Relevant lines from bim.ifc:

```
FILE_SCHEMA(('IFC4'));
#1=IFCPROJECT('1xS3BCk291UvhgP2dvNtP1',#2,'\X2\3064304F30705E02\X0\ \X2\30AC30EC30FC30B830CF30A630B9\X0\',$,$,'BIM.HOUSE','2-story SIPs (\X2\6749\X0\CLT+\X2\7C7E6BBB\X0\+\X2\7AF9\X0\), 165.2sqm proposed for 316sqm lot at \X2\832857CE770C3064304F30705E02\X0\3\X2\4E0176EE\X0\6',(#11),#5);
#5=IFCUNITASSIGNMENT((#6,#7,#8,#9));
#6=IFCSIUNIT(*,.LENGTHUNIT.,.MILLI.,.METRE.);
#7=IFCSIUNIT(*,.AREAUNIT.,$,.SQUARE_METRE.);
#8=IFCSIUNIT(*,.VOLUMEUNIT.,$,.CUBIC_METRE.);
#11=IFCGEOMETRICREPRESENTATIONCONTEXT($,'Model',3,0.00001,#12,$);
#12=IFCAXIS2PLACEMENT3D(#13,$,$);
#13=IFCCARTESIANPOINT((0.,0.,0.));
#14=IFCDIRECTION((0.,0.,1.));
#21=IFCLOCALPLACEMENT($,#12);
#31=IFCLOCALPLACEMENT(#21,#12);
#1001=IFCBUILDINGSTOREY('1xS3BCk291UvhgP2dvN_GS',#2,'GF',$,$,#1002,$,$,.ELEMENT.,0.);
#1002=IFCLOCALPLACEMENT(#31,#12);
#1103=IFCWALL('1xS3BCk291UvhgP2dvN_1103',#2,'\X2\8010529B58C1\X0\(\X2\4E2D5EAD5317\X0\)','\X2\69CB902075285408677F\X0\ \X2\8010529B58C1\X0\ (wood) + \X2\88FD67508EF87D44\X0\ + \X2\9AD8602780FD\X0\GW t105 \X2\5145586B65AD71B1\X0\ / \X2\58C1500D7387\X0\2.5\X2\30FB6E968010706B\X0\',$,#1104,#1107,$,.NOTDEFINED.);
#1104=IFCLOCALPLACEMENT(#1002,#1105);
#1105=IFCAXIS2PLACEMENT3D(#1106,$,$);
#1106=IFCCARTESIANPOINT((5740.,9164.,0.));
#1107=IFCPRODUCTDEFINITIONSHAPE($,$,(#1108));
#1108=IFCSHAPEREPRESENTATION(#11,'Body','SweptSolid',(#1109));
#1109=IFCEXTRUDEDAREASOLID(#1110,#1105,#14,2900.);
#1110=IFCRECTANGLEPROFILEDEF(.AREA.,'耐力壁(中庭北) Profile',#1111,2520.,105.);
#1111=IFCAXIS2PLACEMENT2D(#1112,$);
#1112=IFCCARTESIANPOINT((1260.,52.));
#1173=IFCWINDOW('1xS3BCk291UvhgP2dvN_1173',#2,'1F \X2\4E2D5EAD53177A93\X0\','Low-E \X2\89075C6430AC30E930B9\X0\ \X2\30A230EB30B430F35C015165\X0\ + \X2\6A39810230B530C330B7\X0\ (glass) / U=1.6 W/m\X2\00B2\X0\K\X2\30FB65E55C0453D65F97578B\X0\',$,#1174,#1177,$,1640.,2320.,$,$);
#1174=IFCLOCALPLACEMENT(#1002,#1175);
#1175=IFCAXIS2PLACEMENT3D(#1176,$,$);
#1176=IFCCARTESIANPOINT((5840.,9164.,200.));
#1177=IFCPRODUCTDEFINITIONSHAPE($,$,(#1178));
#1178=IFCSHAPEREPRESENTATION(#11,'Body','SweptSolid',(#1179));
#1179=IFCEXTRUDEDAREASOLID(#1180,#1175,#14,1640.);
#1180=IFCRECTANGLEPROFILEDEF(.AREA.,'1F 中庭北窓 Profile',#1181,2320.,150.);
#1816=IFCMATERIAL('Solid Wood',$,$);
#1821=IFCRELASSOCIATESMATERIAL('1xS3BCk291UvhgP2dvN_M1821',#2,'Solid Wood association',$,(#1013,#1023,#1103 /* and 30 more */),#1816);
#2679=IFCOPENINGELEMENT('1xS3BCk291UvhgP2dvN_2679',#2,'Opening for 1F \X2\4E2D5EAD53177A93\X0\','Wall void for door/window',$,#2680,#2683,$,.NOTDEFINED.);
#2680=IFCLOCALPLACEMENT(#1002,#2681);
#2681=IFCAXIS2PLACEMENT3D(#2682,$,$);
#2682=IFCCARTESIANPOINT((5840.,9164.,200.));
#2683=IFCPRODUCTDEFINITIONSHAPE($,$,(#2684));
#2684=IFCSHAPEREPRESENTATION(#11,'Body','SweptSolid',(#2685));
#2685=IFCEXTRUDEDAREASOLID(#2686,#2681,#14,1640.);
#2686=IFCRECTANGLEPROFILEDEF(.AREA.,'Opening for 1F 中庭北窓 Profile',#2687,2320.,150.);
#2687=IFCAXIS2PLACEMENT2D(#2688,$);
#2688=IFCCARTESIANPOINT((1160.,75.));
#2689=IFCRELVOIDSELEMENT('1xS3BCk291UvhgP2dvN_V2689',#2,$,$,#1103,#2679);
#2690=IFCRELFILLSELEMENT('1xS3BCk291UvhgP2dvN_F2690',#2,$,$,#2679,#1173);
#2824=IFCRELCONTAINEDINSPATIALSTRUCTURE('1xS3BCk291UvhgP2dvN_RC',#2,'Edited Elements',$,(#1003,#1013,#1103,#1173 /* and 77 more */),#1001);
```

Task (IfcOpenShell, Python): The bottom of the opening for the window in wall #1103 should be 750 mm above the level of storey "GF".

```python
import numpy as np
import ifcopenshell
import ifcopenshell.api.geometry
import ifcopenshell.geom
import ifcopenshell.util.element
import ifcopenshell.util.placement
import ifcopenshell.util.shape
import ifcopenshell.util.unit

model = ifcopenshell.open("bim.ifc")
unit_scale = ifcopenshell.util.unit.calculate_unit_scale(model)

window = model.by_guid("1xS3BCk291UvhgP2dvN_1173")
opening = window.FillsVoids[0].RelatingOpeningElement
storey = ifcopenshell.util.element.get_container(window, ifc_class="IfcBuildingStorey")
level = ifcopenshell.util.placement.get_local_placement(storey.ObjectPlacement)[2, 3]

# The opening's origin need not be at the sill, so measure its lowest point.
shape = ifcopenshell.geom.create_shape(ifcopenshell.geom.settings(), opening)
bottom = ifcopenshell.util.shape.get_shape_bottom_elevation(shape, shape.geometry) / unit_scale
dz = level + 750.0 - bottom

shift = np.array([0.0, 0.0, dz])
# The window is not placed relative to its opening, so move both.
for product in (opening, window):
    matrix = ifcopenshell.util.placement.get_local_placement(product.ObjectPlacement)
    matrix[:3, 3] += shift
    ifcopenshell.api.geometry.edit_object_placement(model, product=product, matrix=matrix, is_si=False)

print(f"moved by {dz * unit_scale:+.3f} m")

model.write("bim_rev.ifc")
```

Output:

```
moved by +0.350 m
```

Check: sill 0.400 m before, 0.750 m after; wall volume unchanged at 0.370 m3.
